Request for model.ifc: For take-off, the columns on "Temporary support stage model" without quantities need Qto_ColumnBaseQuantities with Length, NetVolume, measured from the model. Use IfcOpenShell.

First a look at what the model holds.

```python
import ifcopenshell
import ifcopenshell.util.element
import ifcopenshell.util.unit

model = ifcopenshell.open("model.ifc")
print(model.schema)
for unit_type in ("LENGTHUNIT", "AREAUNIT", "VOLUMEUNIT"):
    print(unit_type, ifcopenshell.util.unit.calculate_unit_scale(model, unit_type))
storey = next(s for s in model.by_type("IfcBuildingStorey") if s.Name == "Temporary support stage model")
columns = [e for e in ifcopenshell.util.element.get_decomposition(storey) if e.is_a("IfcColumn")]
for e in sorted(columns, key=lambda e: e.id()):
    print(e.id(), e.is_a(), e.Name, list(ifcopenshell.util.element.get_psets(e, qtos_only=True)), sep=" | ")
```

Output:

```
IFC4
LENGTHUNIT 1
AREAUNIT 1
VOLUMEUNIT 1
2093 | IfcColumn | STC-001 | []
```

```python
import ifcopenshell
import ifcopenshell.api.pset
import ifcopenshell.geom
import ifcopenshell.util.element
import ifcopenshell.util.shape
import ifcopenshell.util.unit

model = ifcopenshell.open("model.ifc")
unit_scale = ifcopenshell.util.unit.calculate_unit_scale(model)
volume_scale = ifcopenshell.util.unit.calculate_unit_scale(model, "VOLUMEUNIT")
settings = ifcopenshell.geom.settings()

storey = next(s for s in model.by_type("IfcBuildingStorey") if s.Name == "Temporary support stage model")
columns = [e for e in ifcopenshell.util.element.get_decomposition(storey) if e.is_a("IfcColumn")]

for e in sorted(columns, key=lambda e: e.id()):
    if ifcopenshell.util.element.get_psets(e, qtos_only=True, should_inherit=False):
        continue
    # Geometry comes back in metres, in the element's own axes.
    shape = ifcopenshell.geom.create_shape(settings, e)
    values = {
        "Length": ifcopenshell.util.shape.get_z(shape.geometry) / unit_scale,
        "NetVolume": ifcopenshell.util.shape.get_volume(shape.geometry) / volume_scale,
    }
    qto = ifcopenshell.api.pset.add_qto(model, product=e, name="Qto_ColumnBaseQuantities")
    ifcopenshell.api.pset.edit_qto(model, qto=qto, properties=values)
    print(e.id(), {k: round(v, 3) for k, v in values.items()})

model.write("model_v2.ifc")
```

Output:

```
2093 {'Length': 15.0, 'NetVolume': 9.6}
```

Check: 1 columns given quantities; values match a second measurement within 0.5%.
